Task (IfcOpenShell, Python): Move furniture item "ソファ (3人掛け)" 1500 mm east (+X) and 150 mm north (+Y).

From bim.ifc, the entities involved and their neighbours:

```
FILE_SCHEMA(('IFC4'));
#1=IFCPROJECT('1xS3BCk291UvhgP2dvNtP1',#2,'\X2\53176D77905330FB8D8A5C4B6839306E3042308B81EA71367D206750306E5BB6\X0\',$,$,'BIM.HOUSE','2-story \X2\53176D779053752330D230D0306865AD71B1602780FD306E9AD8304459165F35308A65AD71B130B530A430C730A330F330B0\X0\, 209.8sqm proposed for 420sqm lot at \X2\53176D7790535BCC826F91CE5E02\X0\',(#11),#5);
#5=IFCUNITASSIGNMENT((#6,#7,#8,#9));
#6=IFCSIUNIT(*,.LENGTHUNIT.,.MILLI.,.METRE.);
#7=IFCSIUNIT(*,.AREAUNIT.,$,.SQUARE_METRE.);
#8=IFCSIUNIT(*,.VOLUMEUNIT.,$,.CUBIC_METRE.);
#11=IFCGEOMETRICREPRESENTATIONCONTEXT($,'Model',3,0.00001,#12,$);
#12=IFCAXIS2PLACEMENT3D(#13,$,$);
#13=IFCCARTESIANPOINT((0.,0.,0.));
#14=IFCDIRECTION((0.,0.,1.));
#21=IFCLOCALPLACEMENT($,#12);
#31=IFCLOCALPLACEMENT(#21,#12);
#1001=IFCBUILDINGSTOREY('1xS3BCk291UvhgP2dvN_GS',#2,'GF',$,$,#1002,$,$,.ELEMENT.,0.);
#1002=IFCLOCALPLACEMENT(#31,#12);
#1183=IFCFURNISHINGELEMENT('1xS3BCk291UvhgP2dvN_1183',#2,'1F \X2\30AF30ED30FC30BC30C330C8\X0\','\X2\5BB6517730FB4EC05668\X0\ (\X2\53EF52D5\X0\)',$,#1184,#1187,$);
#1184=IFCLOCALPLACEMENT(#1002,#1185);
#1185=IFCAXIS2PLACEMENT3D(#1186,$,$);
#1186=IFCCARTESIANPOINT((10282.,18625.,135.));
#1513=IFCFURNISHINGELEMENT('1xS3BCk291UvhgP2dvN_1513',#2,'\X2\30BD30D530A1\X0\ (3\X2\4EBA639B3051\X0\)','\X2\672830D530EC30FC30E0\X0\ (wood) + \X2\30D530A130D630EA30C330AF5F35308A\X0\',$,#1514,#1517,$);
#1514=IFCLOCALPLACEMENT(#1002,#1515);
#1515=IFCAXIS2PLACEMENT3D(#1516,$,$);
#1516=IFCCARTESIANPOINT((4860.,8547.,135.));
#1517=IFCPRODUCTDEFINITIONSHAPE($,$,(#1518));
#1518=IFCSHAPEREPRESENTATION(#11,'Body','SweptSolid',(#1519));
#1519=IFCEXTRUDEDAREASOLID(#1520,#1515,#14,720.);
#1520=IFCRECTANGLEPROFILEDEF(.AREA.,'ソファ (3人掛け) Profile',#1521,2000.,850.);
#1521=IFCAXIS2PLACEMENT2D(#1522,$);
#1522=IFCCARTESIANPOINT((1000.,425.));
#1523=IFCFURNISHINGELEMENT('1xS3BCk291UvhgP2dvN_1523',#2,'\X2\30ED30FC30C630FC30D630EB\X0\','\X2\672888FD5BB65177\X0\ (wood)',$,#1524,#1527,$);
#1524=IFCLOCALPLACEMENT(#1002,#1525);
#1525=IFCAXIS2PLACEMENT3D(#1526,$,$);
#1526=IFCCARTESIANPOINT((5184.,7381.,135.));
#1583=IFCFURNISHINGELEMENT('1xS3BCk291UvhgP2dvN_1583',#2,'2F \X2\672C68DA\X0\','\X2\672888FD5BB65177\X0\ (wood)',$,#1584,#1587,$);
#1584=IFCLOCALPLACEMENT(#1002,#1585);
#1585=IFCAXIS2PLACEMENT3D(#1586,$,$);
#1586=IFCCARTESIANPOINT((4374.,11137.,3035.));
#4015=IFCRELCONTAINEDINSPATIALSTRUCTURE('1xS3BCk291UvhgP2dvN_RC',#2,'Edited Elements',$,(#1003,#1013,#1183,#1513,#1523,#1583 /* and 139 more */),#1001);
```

```python
import ifcopenshell
import ifcopenshell.api.geometry
import ifcopenshell.util.placement

model = ifcopenshell.open("bim.ifc")

item = model.by_guid("1xS3BCk291UvhgP2dvN_1513")
matrix = ifcopenshell.util.placement.get_local_placement(item.ObjectPlacement)
matrix[0, 3] += 1500.0
matrix[1, 3] += 150.0
ifcopenshell.api.geometry.edit_object_placement(model, product=item, matrix=matrix, is_si=False)

print(ifcopenshell.util.placement.get_local_placement(item.ObjectPlacement).round(3) + 0.0)

model.write("bim_edited.ifc")
```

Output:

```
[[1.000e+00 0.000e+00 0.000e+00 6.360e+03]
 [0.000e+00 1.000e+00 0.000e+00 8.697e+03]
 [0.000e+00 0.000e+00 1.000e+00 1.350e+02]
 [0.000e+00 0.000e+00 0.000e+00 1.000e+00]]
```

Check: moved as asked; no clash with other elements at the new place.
